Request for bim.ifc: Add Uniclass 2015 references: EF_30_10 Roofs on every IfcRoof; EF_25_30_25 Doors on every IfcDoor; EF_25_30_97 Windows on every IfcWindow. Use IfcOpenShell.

First a look at what the model holds.

```python
import ifcopenshell

model = ifcopenshell.open("bim.ifc")
print(model.schema)
print("classifications:", [c.Name for c in model.by_type("IfcClassification")])
for ifc_class in ("IfcDoor", "IfcRoof", "IfcStair", "IfcWall", "IfcWindow"):
    print(ifc_class, len(model.by_type(ifc_class)))
```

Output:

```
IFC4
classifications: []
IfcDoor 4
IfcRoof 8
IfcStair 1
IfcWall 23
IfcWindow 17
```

```python
import ifcopenshell
import ifcopenshell.api.classification

model = ifcopenshell.open("bim.ifc")

system = ifcopenshell.api.classification.add_classification(model, classification="Uniclass 2015")

codes = {
    "IfcRoof": ("EF_30_10", "Roofs"),
    "IfcDoor": ("EF_25_30_25", "Doors"),
    "IfcWindow": ("EF_25_30_97", "Windows"),
}
for ifc_class, (code, name) in codes.items():
    products = model.by_type(ifc_class)
    ifcopenshell.api.classification.add_reference(
        model, products=products, classification=system, identification=code, name=name
    )
    print(code, len(products))

model.write("bim_v2.ifc")
```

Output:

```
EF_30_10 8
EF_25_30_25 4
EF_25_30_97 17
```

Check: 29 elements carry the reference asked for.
